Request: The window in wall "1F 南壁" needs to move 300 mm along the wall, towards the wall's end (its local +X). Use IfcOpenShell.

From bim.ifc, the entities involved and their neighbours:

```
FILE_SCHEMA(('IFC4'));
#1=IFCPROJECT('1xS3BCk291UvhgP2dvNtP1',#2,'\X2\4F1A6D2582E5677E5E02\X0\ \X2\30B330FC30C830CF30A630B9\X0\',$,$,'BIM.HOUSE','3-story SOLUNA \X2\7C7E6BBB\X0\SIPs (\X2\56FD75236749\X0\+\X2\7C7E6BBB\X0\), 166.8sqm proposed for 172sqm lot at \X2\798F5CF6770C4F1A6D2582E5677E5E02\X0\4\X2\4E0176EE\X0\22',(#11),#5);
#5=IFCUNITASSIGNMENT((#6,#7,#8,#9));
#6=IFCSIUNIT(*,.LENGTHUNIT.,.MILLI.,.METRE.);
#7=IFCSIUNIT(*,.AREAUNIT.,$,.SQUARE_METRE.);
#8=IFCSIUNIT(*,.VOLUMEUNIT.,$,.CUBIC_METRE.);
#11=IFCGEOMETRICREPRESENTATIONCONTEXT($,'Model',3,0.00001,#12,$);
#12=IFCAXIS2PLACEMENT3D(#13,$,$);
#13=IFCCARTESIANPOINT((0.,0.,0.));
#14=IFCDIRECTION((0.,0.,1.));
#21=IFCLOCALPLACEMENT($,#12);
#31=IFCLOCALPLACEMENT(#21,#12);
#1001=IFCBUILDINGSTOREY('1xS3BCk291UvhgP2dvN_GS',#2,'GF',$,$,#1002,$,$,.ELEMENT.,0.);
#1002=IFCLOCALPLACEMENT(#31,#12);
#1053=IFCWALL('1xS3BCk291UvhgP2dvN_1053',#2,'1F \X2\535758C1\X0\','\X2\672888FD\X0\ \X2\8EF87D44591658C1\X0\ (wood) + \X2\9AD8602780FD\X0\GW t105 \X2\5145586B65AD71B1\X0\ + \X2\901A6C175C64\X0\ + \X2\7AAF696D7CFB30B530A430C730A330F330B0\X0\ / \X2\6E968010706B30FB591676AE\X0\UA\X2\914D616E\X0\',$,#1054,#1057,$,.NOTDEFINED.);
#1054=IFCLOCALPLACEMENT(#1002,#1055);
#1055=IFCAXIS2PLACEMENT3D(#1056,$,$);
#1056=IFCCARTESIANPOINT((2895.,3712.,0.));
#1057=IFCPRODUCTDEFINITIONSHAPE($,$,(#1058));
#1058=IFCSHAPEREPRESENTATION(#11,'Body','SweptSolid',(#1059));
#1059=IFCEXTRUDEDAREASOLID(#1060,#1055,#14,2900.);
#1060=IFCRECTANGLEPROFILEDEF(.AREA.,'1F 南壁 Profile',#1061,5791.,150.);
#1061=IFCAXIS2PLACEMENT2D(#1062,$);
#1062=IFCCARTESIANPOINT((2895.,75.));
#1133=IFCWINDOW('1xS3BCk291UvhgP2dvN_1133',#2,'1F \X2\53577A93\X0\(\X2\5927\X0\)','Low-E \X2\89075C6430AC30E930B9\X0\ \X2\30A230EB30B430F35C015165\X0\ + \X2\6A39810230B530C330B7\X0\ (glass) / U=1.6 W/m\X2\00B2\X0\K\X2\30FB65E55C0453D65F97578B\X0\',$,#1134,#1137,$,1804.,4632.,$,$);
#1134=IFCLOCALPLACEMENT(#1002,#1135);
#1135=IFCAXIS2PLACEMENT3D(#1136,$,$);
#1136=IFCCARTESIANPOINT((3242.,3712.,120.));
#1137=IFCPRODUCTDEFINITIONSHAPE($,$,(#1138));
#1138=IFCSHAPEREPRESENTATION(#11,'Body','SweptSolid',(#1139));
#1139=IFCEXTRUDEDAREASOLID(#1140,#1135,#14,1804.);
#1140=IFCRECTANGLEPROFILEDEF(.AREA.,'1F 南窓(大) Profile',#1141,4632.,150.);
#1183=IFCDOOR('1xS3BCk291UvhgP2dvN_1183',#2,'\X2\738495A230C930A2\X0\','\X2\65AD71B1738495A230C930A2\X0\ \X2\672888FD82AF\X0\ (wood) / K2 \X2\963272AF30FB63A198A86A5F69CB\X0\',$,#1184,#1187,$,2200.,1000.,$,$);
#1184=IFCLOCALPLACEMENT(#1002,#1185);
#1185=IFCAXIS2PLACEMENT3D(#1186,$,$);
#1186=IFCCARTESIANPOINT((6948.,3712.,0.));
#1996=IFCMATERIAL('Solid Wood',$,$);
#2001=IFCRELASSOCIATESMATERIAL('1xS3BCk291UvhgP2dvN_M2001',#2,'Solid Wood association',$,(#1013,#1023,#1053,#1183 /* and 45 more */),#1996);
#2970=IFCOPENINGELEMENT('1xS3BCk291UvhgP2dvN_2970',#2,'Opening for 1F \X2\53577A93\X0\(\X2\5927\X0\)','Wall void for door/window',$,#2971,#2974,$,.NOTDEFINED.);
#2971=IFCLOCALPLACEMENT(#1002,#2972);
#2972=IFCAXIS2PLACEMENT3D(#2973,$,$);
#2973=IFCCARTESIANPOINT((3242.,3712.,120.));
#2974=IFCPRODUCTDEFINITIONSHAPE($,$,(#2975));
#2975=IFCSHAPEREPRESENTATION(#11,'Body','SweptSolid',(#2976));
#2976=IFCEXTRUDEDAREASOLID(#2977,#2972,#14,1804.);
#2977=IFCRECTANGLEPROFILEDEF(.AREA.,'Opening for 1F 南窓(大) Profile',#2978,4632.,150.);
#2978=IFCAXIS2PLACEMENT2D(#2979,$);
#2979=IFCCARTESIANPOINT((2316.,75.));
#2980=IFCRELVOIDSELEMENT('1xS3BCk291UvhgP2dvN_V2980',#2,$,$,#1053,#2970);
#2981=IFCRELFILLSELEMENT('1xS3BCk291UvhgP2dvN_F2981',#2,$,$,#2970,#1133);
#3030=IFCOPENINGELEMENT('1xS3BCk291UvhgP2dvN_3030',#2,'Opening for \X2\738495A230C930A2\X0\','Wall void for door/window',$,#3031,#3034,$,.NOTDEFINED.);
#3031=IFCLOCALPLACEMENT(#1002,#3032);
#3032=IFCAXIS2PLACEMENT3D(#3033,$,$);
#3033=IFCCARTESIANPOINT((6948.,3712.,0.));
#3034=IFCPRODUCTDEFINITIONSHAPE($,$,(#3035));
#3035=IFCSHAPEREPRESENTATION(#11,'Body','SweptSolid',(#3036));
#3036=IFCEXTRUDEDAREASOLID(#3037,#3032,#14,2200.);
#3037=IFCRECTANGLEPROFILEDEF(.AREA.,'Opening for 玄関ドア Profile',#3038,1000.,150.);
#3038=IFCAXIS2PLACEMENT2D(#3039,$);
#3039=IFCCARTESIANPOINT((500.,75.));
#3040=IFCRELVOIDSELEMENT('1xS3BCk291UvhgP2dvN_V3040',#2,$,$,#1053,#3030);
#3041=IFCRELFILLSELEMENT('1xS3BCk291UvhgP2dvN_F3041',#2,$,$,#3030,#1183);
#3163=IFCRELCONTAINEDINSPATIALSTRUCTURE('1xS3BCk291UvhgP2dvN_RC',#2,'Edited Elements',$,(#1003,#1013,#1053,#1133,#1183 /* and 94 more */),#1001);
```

```python
import ifcopenshell
import ifcopenshell.api.geometry
import ifcopenshell.util.placement
import ifcopenshell.util.unit

model = ifcopenshell.open("bim.ifc")
unit_scale = ifcopenshell.util.unit.calculate_unit_scale(model)

window = model.by_guid("1xS3BCk291UvhgP2dvN_1133")
opening = window.FillsVoids[0].RelatingOpeningElement
wall = opening.VoidsElements[0].RelatingBuildingElement

wall_matrix = ifcopenshell.util.placement.get_local_placement(wall.ObjectPlacement)
shift = wall_matrix[:3, 0] * 0.3 / unit_scale
before = ifcopenshell.util.placement.get_local_placement(window.ObjectPlacement)[:3, 3].copy()

# The window is not placed relative to its opening, so move both.
for product in (opening, window):
    matrix = ifcopenshell.util.placement.get_local_placement(product.ObjectPlacement)
    matrix[:3, 3] += shift
    ifcopenshell.api.geometry.edit_object_placement(model, product=product, matrix=matrix, is_si=False)

after = ifcopenshell.util.placement.get_local_placement(window.ObjectPlacement)[:3, 3]
print("window moved by", (after - before).round(3) + 0.0)

model.write("bim-out.ifc")
```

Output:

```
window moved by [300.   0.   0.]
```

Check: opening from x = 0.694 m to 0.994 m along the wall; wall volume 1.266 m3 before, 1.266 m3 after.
